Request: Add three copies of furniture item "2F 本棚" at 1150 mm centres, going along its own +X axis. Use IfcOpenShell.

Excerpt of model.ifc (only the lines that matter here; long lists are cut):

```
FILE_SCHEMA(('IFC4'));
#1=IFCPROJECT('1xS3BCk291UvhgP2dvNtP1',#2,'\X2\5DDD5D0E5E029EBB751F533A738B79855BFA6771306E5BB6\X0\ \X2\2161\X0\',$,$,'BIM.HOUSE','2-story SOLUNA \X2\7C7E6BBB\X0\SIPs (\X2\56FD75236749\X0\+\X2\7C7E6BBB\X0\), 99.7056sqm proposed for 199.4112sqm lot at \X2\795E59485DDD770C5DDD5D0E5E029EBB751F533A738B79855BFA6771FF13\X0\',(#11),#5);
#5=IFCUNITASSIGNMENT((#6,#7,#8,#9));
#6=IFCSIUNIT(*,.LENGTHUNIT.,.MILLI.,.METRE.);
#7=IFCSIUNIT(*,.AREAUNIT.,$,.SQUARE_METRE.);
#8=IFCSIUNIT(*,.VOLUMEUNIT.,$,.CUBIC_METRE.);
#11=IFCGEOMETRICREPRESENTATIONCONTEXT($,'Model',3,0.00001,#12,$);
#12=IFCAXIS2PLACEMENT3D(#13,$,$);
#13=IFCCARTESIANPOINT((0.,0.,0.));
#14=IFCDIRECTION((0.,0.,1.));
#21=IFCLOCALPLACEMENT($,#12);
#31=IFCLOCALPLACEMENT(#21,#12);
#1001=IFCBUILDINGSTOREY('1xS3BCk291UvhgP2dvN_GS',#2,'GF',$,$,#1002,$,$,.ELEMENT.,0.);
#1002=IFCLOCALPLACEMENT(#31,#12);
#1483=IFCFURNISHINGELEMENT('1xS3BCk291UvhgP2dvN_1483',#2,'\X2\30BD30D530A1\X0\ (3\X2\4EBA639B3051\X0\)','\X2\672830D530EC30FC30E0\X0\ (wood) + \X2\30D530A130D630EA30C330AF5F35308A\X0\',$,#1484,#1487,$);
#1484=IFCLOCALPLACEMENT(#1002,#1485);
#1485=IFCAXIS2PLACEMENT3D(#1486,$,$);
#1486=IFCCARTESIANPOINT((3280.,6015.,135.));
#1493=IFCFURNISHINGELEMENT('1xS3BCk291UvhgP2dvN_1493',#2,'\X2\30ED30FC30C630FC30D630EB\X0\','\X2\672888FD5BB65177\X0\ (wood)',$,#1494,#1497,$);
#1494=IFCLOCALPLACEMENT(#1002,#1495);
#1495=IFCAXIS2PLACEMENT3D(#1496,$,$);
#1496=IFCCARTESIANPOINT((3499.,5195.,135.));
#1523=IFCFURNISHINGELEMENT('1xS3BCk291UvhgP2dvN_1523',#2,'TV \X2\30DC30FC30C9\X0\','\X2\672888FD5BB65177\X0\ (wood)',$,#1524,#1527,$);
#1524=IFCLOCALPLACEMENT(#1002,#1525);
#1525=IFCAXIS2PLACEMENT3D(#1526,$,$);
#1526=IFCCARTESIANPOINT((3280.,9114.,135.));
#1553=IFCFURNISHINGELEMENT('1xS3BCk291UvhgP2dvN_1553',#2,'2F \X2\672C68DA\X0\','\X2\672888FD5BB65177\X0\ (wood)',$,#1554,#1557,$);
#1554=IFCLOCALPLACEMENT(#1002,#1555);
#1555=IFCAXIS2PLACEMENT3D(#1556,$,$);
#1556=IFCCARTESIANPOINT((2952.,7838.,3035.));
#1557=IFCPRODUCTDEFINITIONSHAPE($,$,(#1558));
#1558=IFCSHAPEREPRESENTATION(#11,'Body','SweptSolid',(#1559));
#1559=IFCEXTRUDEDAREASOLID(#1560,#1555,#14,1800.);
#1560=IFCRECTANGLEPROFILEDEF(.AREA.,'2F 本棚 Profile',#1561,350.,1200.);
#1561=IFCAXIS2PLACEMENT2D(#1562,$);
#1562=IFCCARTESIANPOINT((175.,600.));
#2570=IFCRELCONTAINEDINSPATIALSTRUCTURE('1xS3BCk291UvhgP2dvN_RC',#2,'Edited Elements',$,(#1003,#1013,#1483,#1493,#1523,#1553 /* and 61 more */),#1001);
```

```python
import ifcopenshell
import ifcopenshell.api.geometry
import ifcopenshell.api.root
import ifcopenshell.util.element
import ifcopenshell.util.placement

model = ifcopenshell.open("model.ifc")


def reuse_history(source, copy):
    """copy_class also copies each property set's owner history, people and application; keep the originals."""
    for rel in copy.IsDefinedBy:
        if rel.is_a("IfcRelDefinesByProperties") and (history := rel.RelatingPropertyDefinition.OwnerHistory):
            rel.RelatingPropertyDefinition.OwnerHistory = source.OwnerHistory
            ifcopenshell.util.element.remove_deep2(model, history)


source = model.by_guid("1xS3BCk291UvhgP2dvN_1553")
base = ifcopenshell.util.placement.get_local_placement(source.ObjectPlacement)
step = base[:3, 0] * 1150.0

for i in range(1, 4):
    copy = ifcopenshell.api.root.copy_class(model, product=source)
    copy.Representation = ifcopenshell.util.element.copy_deep(
        model, source.Representation, exclude=["IfcGeometricRepresentationContext", "IfcRepresentationMap"]
    )
    reuse_history(source, copy)
    matrix = base.copy()
    matrix[:3, 3] += i * step
    print("added at", matrix[:3, 3].round(3) + 0.0)
    ifcopenshell.api.geometry.edit_object_placement(model, product=copy, matrix=matrix, is_si=False)

model.write("model-out.ifc")
```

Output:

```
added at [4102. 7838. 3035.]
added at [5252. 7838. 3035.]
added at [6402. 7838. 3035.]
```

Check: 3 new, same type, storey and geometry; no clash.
